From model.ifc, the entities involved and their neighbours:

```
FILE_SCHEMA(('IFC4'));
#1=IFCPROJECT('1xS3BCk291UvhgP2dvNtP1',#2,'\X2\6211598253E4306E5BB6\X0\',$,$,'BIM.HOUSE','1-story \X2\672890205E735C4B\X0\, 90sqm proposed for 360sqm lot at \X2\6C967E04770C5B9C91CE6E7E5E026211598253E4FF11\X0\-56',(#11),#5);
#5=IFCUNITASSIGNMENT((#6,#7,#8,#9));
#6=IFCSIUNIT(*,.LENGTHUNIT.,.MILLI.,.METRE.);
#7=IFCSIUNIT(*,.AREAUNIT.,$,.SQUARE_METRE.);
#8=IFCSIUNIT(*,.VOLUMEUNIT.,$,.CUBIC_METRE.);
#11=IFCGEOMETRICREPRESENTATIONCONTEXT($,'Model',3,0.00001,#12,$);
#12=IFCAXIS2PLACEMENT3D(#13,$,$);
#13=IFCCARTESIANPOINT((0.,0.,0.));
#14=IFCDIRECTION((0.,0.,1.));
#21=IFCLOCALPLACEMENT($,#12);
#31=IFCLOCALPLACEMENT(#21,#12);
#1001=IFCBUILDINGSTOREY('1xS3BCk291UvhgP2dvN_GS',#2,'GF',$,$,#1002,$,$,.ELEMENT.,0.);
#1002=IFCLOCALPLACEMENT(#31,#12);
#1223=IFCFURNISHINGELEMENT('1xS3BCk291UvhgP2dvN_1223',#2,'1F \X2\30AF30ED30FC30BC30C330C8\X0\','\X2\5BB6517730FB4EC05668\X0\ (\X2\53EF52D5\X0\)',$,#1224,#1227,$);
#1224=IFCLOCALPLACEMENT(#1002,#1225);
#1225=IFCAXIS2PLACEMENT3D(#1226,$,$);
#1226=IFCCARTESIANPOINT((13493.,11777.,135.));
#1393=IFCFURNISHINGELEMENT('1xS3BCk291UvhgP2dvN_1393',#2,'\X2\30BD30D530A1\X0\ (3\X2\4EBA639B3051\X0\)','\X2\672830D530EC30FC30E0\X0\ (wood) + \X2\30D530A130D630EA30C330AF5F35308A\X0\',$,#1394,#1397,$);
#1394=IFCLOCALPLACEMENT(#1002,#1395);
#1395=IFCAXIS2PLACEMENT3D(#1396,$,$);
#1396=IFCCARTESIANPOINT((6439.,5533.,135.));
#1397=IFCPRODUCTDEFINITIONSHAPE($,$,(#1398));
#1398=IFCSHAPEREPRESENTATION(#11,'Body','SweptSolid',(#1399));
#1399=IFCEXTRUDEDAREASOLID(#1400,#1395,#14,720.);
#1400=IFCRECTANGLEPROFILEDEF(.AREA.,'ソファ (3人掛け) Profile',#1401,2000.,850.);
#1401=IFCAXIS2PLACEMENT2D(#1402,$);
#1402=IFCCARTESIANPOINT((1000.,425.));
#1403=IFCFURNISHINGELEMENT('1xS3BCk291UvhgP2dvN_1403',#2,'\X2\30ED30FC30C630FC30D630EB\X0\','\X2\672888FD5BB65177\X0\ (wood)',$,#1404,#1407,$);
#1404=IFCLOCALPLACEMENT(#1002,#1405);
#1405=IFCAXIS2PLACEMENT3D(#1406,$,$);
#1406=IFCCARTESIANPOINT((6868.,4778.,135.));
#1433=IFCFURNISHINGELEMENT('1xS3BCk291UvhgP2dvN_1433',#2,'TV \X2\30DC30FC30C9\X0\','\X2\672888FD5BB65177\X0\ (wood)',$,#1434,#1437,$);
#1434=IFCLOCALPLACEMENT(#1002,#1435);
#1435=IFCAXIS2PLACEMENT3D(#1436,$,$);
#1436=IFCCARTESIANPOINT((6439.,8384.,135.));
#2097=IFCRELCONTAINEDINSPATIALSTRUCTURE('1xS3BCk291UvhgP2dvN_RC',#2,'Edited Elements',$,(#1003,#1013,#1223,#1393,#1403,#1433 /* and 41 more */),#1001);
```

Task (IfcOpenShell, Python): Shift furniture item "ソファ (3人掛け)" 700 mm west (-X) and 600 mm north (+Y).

```python
import ifcopenshell
import ifcopenshell.api.geometry
import ifcopenshell.util.placement

model = ifcopenshell.open("model.ifc")

item = model.by_guid("1xS3BCk291UvhgP2dvN_1393")
matrix = ifcopenshell.util.placement.get_local_placement(item.ObjectPlacement)
matrix[0, 3] -= 700.0
matrix[1, 3] += 600.0
ifcopenshell.api.geometry.edit_object_placement(model, product=item, matrix=matrix, is_si=False)

print(ifcopenshell.util.placement.get_local_placement(item.ObjectPlacement).round(3) + 0.0)

model.write("model_edited.ifc")
```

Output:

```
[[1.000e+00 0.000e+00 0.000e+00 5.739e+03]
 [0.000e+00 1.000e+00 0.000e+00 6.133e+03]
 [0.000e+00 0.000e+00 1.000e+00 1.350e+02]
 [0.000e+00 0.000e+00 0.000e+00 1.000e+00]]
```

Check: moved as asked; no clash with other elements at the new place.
